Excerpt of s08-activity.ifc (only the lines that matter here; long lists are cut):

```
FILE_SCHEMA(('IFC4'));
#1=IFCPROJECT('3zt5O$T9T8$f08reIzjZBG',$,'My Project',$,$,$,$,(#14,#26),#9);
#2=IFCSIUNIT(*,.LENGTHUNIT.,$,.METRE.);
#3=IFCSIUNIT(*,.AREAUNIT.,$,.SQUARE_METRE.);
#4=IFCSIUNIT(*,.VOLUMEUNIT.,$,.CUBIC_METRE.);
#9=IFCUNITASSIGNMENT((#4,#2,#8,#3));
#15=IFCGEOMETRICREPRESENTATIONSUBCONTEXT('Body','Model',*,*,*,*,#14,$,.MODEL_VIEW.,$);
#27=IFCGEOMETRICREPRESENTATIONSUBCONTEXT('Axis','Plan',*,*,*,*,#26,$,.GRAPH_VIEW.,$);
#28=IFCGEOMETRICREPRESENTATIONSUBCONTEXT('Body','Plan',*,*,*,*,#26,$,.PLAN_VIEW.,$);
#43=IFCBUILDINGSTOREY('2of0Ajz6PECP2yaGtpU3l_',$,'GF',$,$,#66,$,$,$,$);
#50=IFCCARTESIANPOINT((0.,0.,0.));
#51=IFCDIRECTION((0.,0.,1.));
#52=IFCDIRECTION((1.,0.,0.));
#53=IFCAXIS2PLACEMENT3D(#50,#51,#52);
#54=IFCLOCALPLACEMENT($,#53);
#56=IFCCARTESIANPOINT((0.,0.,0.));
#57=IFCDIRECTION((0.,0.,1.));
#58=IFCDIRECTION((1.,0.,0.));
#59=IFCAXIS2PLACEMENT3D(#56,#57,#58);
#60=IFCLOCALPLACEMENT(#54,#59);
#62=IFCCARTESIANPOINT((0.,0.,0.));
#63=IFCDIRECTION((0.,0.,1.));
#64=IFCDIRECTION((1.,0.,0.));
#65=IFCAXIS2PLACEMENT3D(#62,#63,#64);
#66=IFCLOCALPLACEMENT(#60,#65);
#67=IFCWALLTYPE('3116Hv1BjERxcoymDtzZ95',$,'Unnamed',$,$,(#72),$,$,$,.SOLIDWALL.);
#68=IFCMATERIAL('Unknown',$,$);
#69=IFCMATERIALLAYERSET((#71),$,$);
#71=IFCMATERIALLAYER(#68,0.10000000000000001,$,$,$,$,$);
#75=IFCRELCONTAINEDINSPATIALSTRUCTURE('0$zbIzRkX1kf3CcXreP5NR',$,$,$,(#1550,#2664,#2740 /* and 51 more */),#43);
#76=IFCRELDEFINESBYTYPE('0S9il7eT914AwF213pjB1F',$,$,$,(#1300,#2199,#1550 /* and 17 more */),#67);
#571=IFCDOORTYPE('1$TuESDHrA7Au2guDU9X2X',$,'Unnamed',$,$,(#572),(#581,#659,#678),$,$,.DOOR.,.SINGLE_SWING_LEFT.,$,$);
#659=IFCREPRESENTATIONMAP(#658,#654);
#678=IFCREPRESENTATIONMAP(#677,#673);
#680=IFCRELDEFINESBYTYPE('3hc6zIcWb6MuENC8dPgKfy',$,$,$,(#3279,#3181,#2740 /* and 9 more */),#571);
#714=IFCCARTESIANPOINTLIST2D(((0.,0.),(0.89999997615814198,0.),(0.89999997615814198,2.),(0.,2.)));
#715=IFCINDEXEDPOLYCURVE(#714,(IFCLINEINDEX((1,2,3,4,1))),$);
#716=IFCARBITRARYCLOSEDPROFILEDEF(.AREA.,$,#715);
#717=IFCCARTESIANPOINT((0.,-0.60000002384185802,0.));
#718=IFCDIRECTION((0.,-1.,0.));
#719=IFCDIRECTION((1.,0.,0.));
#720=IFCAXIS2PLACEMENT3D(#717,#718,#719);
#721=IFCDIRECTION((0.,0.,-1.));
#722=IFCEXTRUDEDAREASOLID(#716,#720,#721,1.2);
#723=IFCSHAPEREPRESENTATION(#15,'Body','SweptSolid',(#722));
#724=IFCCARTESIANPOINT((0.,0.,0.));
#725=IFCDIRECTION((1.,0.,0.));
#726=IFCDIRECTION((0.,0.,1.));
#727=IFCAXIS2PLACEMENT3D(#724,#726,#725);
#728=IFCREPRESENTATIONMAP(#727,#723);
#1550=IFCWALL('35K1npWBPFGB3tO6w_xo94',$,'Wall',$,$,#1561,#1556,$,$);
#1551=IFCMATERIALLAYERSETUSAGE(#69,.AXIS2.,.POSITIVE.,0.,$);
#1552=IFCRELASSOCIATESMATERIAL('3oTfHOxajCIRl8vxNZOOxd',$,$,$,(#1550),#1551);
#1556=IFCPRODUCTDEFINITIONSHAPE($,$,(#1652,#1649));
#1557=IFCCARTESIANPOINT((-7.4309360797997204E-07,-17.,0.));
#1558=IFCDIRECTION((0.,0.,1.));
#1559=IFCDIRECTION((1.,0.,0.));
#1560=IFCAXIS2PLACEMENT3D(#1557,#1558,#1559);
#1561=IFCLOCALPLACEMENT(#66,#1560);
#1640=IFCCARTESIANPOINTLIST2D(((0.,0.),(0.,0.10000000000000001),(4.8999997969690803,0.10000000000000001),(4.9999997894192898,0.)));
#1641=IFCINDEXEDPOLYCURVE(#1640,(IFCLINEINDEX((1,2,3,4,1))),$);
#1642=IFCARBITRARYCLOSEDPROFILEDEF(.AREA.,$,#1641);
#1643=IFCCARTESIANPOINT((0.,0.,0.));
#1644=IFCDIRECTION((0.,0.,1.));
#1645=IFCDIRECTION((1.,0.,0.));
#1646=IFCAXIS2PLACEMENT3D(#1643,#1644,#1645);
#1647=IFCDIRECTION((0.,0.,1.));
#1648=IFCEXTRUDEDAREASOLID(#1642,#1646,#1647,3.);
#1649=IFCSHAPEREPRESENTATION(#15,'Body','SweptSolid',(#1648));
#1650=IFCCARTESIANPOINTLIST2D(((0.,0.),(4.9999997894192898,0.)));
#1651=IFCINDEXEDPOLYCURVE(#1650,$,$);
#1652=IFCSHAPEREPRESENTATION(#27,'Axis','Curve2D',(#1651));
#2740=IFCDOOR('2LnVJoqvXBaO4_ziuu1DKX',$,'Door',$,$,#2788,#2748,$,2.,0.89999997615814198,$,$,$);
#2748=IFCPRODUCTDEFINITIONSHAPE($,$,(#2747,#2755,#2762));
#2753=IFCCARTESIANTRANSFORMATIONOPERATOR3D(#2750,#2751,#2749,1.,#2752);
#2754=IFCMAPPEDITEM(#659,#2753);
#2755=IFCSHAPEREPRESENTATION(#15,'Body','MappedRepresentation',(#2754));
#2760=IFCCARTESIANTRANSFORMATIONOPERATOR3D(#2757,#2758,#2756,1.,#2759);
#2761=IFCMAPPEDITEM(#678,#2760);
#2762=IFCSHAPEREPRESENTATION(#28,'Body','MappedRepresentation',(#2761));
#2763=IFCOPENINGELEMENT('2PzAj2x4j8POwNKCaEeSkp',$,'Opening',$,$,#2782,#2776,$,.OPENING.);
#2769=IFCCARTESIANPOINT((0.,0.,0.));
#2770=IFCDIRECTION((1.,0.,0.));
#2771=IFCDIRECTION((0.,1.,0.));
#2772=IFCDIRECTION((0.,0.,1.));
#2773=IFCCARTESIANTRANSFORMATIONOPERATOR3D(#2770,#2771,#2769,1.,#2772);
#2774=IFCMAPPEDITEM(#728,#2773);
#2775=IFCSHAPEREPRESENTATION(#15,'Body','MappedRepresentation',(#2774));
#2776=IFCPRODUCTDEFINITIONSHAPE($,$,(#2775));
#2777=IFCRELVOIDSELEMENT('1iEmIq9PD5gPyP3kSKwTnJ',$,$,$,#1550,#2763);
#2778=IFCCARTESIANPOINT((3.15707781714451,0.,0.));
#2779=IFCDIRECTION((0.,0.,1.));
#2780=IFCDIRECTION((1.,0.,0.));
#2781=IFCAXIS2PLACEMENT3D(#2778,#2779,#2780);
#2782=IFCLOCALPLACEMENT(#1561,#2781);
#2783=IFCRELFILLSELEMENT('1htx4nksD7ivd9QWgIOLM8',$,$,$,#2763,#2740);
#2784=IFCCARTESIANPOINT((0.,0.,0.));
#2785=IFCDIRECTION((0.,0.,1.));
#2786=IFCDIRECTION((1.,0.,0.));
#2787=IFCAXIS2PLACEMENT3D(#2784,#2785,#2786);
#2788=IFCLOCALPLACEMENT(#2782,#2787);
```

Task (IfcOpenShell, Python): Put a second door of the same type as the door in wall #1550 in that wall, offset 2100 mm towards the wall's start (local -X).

```python
import ifcopenshell
import ifcopenshell.api.feature
import ifcopenshell.api.geometry
import ifcopenshell.api.root
import ifcopenshell.geom
import ifcopenshell.util.element
import ifcopenshell.util.placement
import ifcopenshell.util.shape

model = ifcopenshell.open("s08-activity.ifc")
settings = ifcopenshell.geom.settings()


def volume(element):
    """Net volume in cubic metres, openings subtracted."""
    shape = ifcopenshell.geom.create_shape(settings, element)
    return ifcopenshell.util.shape.get_volume(shape.geometry)


door = model.by_id(2740)
opening = door.FillsVoids[0].RelatingOpeningElement
wall = opening.VoidsElements[0].RelatingBuildingElement
before = volume(wall)
shift = ifcopenshell.util.placement.get_local_placement(wall.ObjectPlacement)[:3, 0] * -2.1

# copy_class copies the void relationship, type, container and properties, but no geometry.
new_opening = ifcopenshell.api.root.copy_class(model, product=opening)
new_opening.Representation = ifcopenshell.util.element.copy_deep(
    model, opening.Representation, exclude=["IfcGeometricRepresentationContext", "IfcRepresentationMap"]
)
new_door = ifcopenshell.api.root.copy_class(model, product=door)
new_door.Representation = ifcopenshell.util.element.copy_deep(
    model, door.Representation, exclude=["IfcGeometricRepresentationContext", "IfcRepresentationMap"]
)
ifcopenshell.api.feature.add_filling(model, opening=new_opening, element=new_door)

for old, new in ((opening, new_opening), (door, new_door)):
    matrix = ifcopenshell.util.placement.get_local_placement(old.ObjectPlacement)
    matrix[:3, 3] += shift
    ifcopenshell.api.geometry.edit_object_placement(model, product=new, matrix=matrix, is_si=False)

after = volume(wall)

print(f"wall volume {before:.3f} -> {after:.3f} m3")

model.write("s08-activity-out.ifc")
```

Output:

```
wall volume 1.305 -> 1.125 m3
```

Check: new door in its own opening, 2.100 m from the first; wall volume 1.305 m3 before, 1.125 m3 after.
